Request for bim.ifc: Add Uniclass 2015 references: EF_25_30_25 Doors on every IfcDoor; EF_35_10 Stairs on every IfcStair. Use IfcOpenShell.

First a look at what the model holds.

```python
import ifcopenshell

model = ifcopenshell.open("bim.ifc")
print(model.schema)
print("classifications:", [c.Name for c in model.by_type("IfcClassification")])
for ifc_class in ("IfcDoor", "IfcRoof", "IfcStair", "IfcWall", "IfcWindow"):
    print(ifc_class, len(model.by_type(ifc_class)))
```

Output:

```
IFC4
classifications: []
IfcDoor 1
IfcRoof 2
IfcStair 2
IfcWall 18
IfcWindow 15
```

```python
import ifcopenshell
import ifcopenshell.api.classification

model = ifcopenshell.open("bim.ifc")

system = ifcopenshell.api.classification.add_classification(model, classification="Uniclass 2015")

codes = {
    "IfcDoor": ("EF_25_30_25", "Doors"),
    "IfcStair": ("EF_35_10", "Stairs"),
}
for ifc_class, (code, name) in codes.items():
    products = model.by_type(ifc_class)
    ifcopenshell.api.classification.add_reference(
        model, products=products, classification=system, identification=code, name=name
    )
    print(code, len(products))

model.write("bim_updated.ifc")
```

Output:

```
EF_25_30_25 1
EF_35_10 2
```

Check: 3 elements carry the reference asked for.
